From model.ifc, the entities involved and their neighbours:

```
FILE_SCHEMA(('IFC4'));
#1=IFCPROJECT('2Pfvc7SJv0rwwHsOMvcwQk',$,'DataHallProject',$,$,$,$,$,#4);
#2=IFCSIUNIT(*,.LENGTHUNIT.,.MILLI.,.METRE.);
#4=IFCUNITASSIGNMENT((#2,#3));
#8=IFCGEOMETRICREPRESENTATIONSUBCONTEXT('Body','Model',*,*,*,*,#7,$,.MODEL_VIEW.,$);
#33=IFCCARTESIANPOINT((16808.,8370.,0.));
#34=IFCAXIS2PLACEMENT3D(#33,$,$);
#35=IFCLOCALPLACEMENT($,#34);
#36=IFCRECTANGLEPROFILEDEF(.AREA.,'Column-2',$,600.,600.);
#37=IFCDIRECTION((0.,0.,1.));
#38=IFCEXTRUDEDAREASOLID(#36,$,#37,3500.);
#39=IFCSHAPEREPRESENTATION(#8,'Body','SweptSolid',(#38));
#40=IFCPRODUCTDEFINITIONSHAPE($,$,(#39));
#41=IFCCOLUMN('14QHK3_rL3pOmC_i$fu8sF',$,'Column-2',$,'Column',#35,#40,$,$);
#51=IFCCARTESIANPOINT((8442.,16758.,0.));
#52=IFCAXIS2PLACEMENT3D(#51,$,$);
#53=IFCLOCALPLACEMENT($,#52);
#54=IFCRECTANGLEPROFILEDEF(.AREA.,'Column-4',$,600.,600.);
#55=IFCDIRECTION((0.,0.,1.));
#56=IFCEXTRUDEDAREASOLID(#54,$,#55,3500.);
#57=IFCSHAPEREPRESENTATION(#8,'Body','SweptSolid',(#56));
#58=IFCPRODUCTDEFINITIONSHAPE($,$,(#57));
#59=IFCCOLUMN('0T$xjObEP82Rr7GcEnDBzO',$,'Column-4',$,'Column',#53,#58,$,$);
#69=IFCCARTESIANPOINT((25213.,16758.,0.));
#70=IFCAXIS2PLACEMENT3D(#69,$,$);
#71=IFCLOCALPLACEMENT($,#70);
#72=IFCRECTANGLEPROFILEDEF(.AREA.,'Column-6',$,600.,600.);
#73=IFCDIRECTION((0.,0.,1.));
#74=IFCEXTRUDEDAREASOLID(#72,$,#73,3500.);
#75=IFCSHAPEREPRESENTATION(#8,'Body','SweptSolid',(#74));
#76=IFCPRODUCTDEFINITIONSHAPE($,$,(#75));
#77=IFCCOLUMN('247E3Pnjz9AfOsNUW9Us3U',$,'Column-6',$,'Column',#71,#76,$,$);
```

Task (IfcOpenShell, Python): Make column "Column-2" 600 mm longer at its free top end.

```python
import ifcopenshell
import ifcopenshell.util.representation

model = ifcopenshell.open("model.ifc")

member = model.by_guid("14QHK3_rL3pOmC_i$fu8sF")
change = 600.0

# The extrusion runs towards the end named, so only its depth changes.
body = ifcopenshell.util.representation.get_representation(member, "Model", "Body")
solid = body.Items[0]
old_length = solid.Depth
solid.Depth += change

print(f"length {old_length:g} -> {solid.Depth:g}")

model.write("model_edited.ifc")
```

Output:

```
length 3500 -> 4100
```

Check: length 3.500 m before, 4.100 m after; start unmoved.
